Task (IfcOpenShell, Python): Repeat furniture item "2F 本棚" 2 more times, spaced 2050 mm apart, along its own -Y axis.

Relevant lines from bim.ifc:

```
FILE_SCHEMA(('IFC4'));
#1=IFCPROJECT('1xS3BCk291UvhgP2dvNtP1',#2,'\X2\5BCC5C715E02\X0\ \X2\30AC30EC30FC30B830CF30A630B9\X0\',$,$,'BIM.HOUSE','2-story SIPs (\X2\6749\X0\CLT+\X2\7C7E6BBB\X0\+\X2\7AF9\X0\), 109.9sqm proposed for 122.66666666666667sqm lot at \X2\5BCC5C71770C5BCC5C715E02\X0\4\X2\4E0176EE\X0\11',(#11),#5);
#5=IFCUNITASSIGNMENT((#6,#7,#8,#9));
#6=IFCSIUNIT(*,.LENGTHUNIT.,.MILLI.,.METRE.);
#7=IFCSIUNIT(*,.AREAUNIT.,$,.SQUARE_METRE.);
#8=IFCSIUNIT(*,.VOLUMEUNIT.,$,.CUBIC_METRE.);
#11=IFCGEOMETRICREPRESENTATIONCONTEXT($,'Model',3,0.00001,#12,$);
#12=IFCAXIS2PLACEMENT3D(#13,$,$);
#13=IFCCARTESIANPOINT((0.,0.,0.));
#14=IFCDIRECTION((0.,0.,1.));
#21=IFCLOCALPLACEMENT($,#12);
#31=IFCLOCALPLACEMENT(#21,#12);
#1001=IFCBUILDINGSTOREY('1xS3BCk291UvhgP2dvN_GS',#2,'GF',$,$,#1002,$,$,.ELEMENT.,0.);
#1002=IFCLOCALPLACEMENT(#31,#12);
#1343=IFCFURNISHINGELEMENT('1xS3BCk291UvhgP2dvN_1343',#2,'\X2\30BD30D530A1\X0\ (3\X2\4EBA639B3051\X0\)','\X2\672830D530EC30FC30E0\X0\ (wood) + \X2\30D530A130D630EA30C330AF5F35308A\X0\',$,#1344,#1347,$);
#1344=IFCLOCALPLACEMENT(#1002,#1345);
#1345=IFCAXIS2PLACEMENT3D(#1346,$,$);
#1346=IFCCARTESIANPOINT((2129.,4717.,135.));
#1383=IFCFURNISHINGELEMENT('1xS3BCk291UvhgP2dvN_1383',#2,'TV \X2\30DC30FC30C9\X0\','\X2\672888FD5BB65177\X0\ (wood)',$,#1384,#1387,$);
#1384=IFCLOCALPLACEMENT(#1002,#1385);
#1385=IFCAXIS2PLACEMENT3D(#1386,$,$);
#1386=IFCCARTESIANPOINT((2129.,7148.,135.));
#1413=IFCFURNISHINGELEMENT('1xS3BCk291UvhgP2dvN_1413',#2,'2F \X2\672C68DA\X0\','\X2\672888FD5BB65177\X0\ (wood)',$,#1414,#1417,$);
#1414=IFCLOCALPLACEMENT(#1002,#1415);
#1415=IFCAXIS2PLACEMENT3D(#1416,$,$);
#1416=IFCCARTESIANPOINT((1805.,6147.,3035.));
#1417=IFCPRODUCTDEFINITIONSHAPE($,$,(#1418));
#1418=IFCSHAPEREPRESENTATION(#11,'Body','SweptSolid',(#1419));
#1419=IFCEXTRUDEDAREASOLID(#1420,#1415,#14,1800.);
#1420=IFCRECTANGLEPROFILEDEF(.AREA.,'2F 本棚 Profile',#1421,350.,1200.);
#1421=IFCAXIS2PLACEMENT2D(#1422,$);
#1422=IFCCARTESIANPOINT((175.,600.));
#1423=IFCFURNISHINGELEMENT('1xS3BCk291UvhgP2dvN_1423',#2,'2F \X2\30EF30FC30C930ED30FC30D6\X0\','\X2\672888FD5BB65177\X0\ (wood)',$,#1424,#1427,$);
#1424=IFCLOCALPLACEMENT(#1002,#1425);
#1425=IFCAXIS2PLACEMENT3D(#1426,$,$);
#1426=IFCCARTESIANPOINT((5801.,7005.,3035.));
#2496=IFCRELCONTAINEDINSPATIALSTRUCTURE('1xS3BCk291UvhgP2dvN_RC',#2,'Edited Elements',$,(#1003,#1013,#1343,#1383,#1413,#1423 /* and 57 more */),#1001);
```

```python
import ifcopenshell
import ifcopenshell.api.geometry
import ifcopenshell.api.root
import ifcopenshell.util.element
import ifcopenshell.util.placement
import ifcopenshell.util.unit

model = ifcopenshell.open("bim.ifc")
unit_scale = ifcopenshell.util.unit.calculate_unit_scale(model)


def reuse_history(source, copy):
    """copy_class also copies each property set's owner history, people and application; keep the originals."""
    for rel in copy.IsDefinedBy:
        if rel.is_a("IfcRelDefinesByProperties") and (history := rel.RelatingPropertyDefinition.OwnerHistory):
            rel.RelatingPropertyDefinition.OwnerHistory = source.OwnerHistory
            ifcopenshell.util.element.remove_deep2(model, history)


source = model.by_id(1413)
base = ifcopenshell.util.placement.get_local_placement(source.ObjectPlacement)
step = -base[:3, 1] * 2.05 / unit_scale

for i in range(1, 3):
    copy = ifcopenshell.api.root.copy_class(model, product=source)
    copy.Representation = ifcopenshell.util.element.copy_deep(
        model, source.Representation, exclude=["IfcGeometricRepresentationContext", "IfcRepresentationMap"]
    )
    reuse_history(source, copy)
    matrix = base.copy()
    matrix[:3, 3] += i * step
    print("added at", matrix[:3, 3].round(3) + 0.0)
    ifcopenshell.api.geometry.edit_object_placement(model, product=copy, matrix=matrix, is_si=False)

model.write("bim-out.ifc")
```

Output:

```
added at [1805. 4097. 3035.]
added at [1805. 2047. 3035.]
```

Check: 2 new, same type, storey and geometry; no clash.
